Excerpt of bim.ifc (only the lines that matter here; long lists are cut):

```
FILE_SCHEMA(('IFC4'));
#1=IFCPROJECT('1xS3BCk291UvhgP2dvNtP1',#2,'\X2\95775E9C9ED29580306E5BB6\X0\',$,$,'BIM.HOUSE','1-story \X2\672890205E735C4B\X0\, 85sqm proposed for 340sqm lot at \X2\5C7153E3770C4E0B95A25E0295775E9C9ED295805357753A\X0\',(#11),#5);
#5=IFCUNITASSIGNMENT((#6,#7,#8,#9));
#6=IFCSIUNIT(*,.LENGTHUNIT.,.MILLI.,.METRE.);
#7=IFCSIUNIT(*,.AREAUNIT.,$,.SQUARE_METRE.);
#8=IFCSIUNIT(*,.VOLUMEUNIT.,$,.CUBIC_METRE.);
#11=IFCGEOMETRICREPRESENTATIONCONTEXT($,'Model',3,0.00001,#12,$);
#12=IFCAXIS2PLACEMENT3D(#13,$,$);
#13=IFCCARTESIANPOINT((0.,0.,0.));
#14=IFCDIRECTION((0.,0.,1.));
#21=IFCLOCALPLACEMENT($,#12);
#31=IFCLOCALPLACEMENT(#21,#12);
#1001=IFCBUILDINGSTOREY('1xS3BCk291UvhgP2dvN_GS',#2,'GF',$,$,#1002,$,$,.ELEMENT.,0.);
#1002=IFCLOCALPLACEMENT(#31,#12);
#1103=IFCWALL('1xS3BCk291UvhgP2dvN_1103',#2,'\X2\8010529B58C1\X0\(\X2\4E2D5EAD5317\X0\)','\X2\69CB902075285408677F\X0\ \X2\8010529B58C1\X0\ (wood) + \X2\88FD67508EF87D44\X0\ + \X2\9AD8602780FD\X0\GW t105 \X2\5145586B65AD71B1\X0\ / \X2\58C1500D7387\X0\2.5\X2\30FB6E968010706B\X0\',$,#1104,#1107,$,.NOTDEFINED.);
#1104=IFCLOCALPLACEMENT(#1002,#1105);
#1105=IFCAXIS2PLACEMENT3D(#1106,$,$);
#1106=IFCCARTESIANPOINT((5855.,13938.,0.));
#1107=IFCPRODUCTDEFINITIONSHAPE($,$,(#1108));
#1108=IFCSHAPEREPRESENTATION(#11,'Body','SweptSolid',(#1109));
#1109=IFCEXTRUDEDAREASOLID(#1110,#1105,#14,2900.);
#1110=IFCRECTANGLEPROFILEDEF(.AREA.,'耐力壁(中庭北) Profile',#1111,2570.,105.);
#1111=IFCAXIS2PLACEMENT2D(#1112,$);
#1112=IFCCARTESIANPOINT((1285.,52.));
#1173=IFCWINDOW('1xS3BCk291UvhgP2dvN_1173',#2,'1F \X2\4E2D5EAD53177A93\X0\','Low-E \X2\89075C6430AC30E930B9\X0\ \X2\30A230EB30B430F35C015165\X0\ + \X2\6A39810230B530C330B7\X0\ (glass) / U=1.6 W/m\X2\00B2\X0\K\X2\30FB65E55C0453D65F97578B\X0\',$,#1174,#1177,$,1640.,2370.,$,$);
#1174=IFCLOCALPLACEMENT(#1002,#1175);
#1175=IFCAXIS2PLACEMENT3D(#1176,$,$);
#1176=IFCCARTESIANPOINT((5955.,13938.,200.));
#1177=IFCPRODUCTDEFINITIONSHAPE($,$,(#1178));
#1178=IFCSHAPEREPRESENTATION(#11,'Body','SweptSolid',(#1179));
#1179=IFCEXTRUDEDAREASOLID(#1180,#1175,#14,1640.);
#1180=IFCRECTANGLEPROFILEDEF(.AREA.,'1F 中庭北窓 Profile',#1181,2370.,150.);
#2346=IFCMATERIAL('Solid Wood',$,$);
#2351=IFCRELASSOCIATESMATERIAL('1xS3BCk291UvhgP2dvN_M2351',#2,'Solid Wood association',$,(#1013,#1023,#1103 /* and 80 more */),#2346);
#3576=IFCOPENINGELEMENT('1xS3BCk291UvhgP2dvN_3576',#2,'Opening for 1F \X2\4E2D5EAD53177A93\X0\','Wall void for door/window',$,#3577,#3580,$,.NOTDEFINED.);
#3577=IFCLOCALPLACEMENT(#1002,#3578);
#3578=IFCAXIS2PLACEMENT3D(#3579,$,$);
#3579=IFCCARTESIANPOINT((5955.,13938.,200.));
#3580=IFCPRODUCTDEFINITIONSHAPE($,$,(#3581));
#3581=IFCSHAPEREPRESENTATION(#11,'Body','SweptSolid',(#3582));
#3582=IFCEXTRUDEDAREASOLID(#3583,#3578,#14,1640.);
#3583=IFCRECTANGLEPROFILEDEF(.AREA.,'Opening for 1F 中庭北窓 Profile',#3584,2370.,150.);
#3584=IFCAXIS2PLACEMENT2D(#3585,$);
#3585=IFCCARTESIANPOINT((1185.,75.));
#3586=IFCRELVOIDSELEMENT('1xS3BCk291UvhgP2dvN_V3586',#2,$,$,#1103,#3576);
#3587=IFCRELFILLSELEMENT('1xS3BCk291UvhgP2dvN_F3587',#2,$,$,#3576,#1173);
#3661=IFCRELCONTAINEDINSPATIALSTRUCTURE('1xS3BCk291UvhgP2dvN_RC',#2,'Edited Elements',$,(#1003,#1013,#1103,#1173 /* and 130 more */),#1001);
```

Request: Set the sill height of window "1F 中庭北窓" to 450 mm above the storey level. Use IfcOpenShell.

```python
import numpy as np
import ifcopenshell
import ifcopenshell.api.geometry
import ifcopenshell.geom
import ifcopenshell.util.element
import ifcopenshell.util.placement
import ifcopenshell.util.shape
import ifcopenshell.util.unit

model = ifcopenshell.open("bim.ifc")
unit_scale = ifcopenshell.util.unit.calculate_unit_scale(model)

window = model.by_id(1173)
opening = window.FillsVoids[0].RelatingOpeningElement
storey = ifcopenshell.util.element.get_container(window, ifc_class="IfcBuildingStorey")
level = ifcopenshell.util.placement.get_local_placement(storey.ObjectPlacement)[2, 3]

# The opening's origin need not be at the sill, so measure its lowest point.
shape = ifcopenshell.geom.create_shape(ifcopenshell.geom.settings(), opening)
bottom = ifcopenshell.util.shape.get_shape_bottom_elevation(shape, shape.geometry) / unit_scale
dz = level + 0.45 / unit_scale - bottom

shift = np.array([0.0, 0.0, dz])
# The window is not placed relative to its opening, so move both.
for product in (opening, window):
    matrix = ifcopenshell.util.placement.get_local_placement(product.ObjectPlacement)
    matrix[:3, 3] += shift
    ifcopenshell.api.geometry.edit_object_placement(model, product=product, matrix=matrix, is_si=False)

print(f"moved by {dz * unit_scale:+.3f} m")

model.write("bim_edited.ifc")
```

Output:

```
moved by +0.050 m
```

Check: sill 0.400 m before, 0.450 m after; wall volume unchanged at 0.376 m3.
